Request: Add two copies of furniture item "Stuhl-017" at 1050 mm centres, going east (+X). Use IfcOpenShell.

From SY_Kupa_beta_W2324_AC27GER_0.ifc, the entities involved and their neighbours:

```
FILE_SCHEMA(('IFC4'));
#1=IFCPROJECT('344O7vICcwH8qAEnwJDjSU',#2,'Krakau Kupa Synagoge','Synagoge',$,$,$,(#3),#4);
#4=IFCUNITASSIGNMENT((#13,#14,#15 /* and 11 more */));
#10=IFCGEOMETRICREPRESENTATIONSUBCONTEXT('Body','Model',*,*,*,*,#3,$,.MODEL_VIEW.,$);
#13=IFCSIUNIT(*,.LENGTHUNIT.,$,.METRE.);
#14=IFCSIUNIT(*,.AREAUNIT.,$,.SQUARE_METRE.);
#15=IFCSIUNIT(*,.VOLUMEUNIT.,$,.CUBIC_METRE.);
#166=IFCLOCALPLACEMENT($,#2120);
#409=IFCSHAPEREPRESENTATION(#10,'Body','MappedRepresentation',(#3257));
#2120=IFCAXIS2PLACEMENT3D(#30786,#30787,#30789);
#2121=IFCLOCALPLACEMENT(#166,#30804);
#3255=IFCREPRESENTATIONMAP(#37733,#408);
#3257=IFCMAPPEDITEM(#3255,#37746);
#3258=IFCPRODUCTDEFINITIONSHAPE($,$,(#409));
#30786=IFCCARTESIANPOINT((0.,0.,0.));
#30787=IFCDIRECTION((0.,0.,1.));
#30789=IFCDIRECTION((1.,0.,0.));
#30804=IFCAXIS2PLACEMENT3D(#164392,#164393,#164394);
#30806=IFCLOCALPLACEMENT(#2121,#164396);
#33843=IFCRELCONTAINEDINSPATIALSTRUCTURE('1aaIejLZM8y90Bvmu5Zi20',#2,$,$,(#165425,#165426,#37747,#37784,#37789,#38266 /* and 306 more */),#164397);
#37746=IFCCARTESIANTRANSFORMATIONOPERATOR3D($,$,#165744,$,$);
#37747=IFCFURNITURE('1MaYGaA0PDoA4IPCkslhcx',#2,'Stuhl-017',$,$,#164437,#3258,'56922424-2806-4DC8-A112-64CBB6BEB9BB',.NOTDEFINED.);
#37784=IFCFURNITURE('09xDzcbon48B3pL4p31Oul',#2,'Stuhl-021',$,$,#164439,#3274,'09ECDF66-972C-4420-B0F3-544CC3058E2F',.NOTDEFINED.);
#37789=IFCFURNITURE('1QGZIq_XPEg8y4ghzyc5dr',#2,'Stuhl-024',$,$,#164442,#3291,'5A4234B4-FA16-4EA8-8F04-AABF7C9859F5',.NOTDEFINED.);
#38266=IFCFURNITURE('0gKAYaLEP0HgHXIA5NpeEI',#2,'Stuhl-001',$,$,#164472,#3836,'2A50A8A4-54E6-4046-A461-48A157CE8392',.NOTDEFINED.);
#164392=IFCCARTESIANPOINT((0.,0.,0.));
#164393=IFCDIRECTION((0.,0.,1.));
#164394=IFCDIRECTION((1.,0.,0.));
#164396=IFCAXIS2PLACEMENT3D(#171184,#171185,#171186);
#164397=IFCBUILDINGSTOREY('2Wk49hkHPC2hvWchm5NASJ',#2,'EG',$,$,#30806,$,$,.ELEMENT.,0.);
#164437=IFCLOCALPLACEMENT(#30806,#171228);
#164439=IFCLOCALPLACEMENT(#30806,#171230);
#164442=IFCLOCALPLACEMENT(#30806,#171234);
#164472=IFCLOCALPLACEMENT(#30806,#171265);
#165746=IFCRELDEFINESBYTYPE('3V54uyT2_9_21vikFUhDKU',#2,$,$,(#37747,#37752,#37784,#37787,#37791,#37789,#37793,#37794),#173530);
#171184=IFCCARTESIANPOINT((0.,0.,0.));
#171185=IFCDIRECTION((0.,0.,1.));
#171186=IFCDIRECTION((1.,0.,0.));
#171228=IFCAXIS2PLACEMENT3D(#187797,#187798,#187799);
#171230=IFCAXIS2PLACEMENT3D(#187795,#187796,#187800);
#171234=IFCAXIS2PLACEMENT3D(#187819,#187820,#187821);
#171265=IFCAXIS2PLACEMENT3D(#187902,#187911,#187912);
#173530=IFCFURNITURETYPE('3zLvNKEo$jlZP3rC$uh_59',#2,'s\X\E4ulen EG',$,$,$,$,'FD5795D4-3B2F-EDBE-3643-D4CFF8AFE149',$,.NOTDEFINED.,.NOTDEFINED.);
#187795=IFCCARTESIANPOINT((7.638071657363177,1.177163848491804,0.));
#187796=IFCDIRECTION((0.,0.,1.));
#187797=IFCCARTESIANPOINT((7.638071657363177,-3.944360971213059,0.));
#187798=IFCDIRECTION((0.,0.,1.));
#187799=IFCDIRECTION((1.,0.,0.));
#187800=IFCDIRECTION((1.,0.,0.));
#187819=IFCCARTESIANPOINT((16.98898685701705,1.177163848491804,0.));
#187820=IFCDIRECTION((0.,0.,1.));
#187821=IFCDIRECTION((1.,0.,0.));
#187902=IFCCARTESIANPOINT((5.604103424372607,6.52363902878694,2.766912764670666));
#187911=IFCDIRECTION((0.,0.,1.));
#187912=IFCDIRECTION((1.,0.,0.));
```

```python
import numpy as np
import ifcopenshell
import ifcopenshell.api.geometry
import ifcopenshell.api.root
import ifcopenshell.util.element
import ifcopenshell.util.placement
import ifcopenshell.util.unit

model = ifcopenshell.open("SY_Kupa_beta_W2324_AC27GER_0.ifc")
unit_scale = ifcopenshell.util.unit.calculate_unit_scale(model)


def reuse_history(source, copy):
    """copy_class also copies each property set's owner history, people and application; keep the originals."""
    for rel in copy.IsDefinedBy:
        if rel.is_a("IfcRelDefinesByProperties") and (history := rel.RelatingPropertyDefinition.OwnerHistory):
            rel.RelatingPropertyDefinition.OwnerHistory = source.OwnerHistory
            ifcopenshell.util.element.remove_deep2(model, history)


source = model.by_guid("1MaYGaA0PDoA4IPCkslhcx")
base = ifcopenshell.util.placement.get_local_placement(source.ObjectPlacement)
step = np.array([1.0, 0.0, 0.0]) * 1.05 / unit_scale

for i in range(1, 3):
    copy = ifcopenshell.api.root.copy_class(model, product=source)
    copy.Representation = ifcopenshell.util.element.copy_deep(
        model, source.Representation, exclude=["IfcGeometricRepresentationContext", "IfcRepresentationMap"]
    )
    copy.Tag = None
    reuse_history(source, copy)
    matrix = base.copy()
    matrix[:3, 3] += i * step
    print("added at", matrix[:3, 3].round(3) + 0.0)
    ifcopenshell.api.geometry.edit_object_placement(model, product=copy, matrix=matrix, is_si=False)

model.write("SY_Kupa_beta_W2324_AC27GER_0_updated.ifc")
```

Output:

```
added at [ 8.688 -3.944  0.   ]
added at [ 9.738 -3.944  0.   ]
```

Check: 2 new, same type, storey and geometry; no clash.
